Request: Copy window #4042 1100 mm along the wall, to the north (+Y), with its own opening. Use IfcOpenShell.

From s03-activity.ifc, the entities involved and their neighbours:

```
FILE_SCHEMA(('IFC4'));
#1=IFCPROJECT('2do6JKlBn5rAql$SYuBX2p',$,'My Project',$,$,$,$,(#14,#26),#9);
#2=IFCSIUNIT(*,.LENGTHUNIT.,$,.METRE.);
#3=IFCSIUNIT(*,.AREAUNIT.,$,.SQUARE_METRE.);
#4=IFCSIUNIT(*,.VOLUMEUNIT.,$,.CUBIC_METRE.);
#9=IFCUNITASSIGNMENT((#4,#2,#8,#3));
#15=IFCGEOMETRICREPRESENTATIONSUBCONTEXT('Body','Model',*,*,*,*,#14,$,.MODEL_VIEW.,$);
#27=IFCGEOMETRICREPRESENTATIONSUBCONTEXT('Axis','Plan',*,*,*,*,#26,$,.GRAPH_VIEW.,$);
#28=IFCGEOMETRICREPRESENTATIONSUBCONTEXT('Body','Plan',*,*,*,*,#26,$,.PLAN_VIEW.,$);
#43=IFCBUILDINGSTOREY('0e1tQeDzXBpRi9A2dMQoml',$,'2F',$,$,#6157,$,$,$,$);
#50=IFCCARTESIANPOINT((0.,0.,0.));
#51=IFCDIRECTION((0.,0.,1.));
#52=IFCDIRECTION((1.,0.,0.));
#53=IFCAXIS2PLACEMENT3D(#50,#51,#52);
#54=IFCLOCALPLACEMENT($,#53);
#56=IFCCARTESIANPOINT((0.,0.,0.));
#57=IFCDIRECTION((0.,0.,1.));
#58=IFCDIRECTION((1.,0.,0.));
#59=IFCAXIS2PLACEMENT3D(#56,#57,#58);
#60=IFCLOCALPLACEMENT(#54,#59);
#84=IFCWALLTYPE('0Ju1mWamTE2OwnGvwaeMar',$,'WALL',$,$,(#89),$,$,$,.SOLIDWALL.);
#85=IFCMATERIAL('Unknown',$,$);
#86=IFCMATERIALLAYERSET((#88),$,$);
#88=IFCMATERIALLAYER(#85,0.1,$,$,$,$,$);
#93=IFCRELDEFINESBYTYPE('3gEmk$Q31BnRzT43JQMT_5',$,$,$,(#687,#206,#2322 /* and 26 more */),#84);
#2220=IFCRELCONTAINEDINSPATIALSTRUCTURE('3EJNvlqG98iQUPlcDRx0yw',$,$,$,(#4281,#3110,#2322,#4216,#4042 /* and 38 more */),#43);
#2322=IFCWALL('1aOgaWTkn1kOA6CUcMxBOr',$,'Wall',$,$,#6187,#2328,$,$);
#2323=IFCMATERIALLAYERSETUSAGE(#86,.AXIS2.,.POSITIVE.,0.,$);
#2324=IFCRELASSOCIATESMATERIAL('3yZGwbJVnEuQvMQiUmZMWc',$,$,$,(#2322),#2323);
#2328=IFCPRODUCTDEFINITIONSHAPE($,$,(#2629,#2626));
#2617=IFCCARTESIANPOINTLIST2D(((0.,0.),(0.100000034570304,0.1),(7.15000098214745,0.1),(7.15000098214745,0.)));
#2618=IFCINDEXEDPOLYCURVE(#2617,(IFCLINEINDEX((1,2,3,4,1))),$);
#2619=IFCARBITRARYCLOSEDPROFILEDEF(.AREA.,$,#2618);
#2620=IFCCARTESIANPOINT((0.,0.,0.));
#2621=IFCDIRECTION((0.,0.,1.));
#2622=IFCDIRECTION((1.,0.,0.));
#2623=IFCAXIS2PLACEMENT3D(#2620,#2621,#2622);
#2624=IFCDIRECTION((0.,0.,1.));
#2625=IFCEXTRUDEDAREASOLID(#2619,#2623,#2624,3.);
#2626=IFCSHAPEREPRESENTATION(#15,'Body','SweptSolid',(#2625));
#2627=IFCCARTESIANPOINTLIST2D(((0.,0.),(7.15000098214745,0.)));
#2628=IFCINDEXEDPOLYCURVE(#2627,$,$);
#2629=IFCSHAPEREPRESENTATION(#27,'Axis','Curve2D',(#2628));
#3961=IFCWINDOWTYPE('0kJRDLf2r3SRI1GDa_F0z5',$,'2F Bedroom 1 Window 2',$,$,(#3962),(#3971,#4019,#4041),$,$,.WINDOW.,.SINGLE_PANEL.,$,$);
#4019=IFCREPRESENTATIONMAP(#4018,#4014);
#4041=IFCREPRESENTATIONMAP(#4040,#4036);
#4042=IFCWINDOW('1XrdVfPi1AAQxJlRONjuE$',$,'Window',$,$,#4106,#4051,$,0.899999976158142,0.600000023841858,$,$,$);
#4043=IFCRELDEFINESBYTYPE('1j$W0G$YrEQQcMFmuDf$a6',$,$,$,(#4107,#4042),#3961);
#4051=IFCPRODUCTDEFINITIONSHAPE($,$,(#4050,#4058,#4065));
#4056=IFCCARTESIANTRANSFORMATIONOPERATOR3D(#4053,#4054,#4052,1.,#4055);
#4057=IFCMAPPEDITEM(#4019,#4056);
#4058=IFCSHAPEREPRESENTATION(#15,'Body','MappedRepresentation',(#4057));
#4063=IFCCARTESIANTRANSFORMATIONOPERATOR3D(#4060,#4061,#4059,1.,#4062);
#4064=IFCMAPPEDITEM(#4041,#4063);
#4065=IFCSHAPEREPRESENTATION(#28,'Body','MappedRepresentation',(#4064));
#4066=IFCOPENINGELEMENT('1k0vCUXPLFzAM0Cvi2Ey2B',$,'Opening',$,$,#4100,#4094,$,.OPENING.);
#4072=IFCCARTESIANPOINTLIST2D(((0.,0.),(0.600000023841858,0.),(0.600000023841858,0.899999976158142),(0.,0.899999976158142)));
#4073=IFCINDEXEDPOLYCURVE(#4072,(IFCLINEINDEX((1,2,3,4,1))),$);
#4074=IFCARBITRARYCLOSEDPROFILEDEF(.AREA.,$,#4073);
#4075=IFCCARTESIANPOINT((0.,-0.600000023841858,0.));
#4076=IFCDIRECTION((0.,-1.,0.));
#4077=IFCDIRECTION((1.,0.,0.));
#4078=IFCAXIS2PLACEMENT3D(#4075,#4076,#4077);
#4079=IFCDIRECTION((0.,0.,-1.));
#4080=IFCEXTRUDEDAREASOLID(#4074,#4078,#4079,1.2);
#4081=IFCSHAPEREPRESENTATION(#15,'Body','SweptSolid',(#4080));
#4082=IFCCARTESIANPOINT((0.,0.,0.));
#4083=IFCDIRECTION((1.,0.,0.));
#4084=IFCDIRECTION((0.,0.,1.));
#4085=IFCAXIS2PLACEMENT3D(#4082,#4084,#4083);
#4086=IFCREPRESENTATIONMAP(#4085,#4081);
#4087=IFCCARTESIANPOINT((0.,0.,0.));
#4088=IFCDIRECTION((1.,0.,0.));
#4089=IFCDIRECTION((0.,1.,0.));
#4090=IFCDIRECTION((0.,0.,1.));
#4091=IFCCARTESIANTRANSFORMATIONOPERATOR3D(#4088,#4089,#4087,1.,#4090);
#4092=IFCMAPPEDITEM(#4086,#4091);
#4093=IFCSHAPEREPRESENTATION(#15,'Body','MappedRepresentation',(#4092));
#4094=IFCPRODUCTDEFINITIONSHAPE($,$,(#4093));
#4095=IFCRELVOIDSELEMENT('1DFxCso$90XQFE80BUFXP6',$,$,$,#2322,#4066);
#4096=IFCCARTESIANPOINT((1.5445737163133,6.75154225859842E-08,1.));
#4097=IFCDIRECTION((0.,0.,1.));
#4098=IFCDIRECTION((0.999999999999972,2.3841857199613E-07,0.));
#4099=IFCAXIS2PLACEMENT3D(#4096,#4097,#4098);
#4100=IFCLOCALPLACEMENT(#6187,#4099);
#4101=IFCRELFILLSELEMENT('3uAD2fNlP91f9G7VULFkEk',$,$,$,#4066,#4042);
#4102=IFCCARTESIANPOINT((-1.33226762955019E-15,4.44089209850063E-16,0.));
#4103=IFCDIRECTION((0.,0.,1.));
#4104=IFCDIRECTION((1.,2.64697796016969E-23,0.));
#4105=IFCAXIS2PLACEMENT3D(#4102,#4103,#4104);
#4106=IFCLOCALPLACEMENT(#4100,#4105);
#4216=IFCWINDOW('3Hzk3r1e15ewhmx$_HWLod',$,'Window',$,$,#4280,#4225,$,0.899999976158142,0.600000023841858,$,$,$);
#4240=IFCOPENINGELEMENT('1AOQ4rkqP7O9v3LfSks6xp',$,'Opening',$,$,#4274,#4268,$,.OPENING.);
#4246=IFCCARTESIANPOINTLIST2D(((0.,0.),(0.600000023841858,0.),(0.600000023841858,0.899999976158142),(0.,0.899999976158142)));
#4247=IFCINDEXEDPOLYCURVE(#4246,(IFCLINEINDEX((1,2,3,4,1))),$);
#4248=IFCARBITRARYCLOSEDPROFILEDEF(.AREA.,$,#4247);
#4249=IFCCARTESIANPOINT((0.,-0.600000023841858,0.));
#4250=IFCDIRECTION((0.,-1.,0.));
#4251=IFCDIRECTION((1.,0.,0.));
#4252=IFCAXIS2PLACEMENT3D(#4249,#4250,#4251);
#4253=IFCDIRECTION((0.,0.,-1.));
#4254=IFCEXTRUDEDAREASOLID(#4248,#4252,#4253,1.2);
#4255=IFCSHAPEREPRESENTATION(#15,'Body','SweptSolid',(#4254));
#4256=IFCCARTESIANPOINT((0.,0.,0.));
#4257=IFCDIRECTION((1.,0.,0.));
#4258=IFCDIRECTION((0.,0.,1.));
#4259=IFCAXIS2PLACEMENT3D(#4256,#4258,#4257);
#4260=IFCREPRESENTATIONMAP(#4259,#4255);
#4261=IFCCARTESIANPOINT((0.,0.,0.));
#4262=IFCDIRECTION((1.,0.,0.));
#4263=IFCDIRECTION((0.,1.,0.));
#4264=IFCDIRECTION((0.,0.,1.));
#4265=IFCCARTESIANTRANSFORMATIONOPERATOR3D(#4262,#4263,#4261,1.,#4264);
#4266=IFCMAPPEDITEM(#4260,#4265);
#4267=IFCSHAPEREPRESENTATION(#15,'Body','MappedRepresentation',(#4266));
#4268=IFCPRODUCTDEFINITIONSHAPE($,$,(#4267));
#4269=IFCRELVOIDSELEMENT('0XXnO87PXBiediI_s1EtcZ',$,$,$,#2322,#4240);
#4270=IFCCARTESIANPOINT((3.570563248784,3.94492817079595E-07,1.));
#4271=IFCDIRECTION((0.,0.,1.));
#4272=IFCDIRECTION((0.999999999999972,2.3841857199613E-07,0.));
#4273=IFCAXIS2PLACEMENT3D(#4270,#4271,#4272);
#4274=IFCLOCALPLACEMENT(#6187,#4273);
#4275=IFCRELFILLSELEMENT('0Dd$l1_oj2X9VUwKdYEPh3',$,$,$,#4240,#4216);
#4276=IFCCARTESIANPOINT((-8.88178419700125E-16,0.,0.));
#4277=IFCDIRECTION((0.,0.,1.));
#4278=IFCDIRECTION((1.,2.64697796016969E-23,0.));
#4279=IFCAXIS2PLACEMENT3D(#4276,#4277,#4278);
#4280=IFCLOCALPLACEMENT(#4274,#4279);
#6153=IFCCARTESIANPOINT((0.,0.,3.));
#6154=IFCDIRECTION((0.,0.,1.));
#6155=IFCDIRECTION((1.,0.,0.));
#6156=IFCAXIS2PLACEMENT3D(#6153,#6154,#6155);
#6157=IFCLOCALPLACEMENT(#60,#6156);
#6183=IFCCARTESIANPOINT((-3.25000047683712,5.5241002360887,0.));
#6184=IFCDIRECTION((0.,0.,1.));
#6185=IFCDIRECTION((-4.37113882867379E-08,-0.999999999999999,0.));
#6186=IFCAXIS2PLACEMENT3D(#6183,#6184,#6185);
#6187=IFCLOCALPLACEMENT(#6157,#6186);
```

```python
import ifcopenshell
import ifcopenshell.api.feature
import ifcopenshell.api.geometry
import ifcopenshell.api.root
import ifcopenshell.geom
import ifcopenshell.util.element
import ifcopenshell.util.placement
import ifcopenshell.util.shape
import ifcopenshell.util.unit

model = ifcopenshell.open("s03-activity.ifc")
unit_scale = ifcopenshell.util.unit.calculate_unit_scale(model)
settings = ifcopenshell.geom.settings()


def volume(element):
    """Net volume in cubic metres, openings subtracted."""
    shape = ifcopenshell.geom.create_shape(settings, element)
    return ifcopenshell.util.shape.get_volume(shape.geometry)


window = model.by_guid("1XrdVfPi1AAQxJlRONjuE$")
opening = window.FillsVoids[0].RelatingOpeningElement
wall = opening.VoidsElements[0].RelatingBuildingElement
before = volume(wall)
shift = ifcopenshell.util.placement.get_local_placement(wall.ObjectPlacement)[:3, 0] * -1.1 / unit_scale

# copy_class copies the void relationship, type, container and properties, but no geometry.
new_opening = ifcopenshell.api.root.copy_class(model, product=opening)
new_opening.Representation = ifcopenshell.util.element.copy_deep(
    model, opening.Representation, exclude=["IfcGeometricRepresentationContext", "IfcRepresentationMap"]
)
new_window = ifcopenshell.api.root.copy_class(model, product=window)
new_window.Representation = ifcopenshell.util.element.copy_deep(
    model, window.Representation, exclude=["IfcGeometricRepresentationContext", "IfcRepresentationMap"]
)
ifcopenshell.api.feature.add_filling(model, opening=new_opening, element=new_window)

for old, new in ((opening, new_opening), (window, new_window)):
    matrix = ifcopenshell.util.placement.get_local_placement(old.ObjectPlacement)
    matrix[:3, 3] += shift
    ifcopenshell.api.geometry.edit_object_placement(model, product=new, matrix=matrix, is_si=False)

after = volume(wall)

print(f"wall volume {before:.3f} -> {after:.3f} m3")

model.write("s03-activity_v2.ifc")
```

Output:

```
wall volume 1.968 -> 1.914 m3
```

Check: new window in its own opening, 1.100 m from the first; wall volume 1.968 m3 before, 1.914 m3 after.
